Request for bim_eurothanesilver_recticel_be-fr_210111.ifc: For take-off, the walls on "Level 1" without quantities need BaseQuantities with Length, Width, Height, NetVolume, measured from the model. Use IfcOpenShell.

First a look at what the model holds.

```python
import ifcopenshell
import ifcopenshell.util.element
import ifcopenshell.util.unit

model = ifcopenshell.open("bim_eurothanesilver_recticel_be-fr_210111.ifc")
print(model.schema)
for unit_type in ("LENGTHUNIT", "AREAUNIT", "VOLUMEUNIT"):
    print(unit_type, ifcopenshell.util.unit.calculate_unit_scale(model, unit_type))
storey = next(s for s in model.by_type("IfcBuildingStorey") if s.Name == "Level 1")
walls = [e for e in ifcopenshell.util.element.get_decomposition(storey) if e.is_a("IfcWall")]
for e in sorted(walls, key=lambda e: e.id()):
    print(e.id(), e.is_a(), e.Name, list(ifcopenshell.util.element.get_psets(e, qtos_only=True)), sep=" | ")
```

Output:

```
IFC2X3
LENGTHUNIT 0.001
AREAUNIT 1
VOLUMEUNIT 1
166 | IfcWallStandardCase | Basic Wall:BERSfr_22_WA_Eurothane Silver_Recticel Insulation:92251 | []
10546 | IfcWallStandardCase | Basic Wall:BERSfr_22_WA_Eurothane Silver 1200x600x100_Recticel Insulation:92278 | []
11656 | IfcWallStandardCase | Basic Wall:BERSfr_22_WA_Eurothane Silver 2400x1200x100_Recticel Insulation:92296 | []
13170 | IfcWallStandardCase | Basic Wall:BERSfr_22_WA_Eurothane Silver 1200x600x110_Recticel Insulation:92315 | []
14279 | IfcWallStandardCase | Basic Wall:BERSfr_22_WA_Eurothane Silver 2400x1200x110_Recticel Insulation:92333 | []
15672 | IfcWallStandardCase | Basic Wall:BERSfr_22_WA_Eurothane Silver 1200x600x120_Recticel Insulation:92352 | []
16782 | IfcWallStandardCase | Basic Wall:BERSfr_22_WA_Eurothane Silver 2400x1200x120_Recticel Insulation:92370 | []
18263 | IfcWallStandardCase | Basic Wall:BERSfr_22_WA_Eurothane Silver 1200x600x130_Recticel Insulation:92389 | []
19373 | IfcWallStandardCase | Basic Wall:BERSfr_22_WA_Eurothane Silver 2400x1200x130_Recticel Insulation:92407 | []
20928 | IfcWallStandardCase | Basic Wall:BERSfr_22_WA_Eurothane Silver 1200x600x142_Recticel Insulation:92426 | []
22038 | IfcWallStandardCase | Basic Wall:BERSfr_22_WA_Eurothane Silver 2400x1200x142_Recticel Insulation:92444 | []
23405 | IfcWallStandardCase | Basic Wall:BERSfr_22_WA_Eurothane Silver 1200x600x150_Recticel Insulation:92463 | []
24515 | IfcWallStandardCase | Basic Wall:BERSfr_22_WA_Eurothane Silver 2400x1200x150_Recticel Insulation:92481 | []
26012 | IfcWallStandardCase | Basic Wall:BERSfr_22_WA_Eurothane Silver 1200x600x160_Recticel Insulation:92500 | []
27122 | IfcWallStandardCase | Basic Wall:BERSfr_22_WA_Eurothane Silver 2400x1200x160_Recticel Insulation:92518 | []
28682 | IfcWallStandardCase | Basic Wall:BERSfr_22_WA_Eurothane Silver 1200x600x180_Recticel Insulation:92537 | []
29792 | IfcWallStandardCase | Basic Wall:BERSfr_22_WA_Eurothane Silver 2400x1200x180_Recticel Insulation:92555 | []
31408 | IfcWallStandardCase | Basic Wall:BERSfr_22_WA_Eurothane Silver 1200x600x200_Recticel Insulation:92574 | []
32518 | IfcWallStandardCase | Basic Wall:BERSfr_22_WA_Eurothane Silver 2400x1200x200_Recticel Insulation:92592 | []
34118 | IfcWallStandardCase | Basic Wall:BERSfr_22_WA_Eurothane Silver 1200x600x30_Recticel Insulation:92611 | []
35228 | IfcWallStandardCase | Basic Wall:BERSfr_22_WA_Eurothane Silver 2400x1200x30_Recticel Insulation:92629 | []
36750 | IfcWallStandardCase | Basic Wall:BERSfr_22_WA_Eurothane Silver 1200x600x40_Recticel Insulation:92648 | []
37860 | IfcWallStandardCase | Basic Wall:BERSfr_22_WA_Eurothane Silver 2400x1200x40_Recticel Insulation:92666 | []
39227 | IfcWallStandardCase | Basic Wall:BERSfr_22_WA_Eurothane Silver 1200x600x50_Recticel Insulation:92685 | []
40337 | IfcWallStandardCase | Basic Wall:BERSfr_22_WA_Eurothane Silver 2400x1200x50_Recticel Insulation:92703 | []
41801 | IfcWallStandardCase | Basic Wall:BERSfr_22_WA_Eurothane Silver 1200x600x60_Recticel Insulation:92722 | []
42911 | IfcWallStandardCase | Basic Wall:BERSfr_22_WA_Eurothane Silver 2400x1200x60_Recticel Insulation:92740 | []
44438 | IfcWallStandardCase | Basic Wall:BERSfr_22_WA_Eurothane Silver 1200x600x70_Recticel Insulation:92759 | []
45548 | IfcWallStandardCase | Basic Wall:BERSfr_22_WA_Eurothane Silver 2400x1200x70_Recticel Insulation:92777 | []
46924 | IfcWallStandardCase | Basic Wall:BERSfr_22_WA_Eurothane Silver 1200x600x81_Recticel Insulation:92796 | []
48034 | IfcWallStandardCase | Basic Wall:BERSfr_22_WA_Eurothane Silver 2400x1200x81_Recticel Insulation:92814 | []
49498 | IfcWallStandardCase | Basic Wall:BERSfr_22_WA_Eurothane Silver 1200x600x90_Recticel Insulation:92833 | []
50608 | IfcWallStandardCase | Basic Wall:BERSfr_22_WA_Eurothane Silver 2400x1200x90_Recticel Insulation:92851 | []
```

```python
import ifcopenshell
import ifcopenshell.api.pset
import ifcopenshell.geom
import ifcopenshell.util.element
import ifcopenshell.util.shape
import ifcopenshell.util.unit

model = ifcopenshell.open("bim_eurothanesilver_recticel_be-fr_210111.ifc")
unit_scale = ifcopenshell.util.unit.calculate_unit_scale(model)
volume_scale = ifcopenshell.util.unit.calculate_unit_scale(model, "VOLUMEUNIT")
settings = ifcopenshell.geom.settings()

storey = next(s for s in model.by_type("IfcBuildingStorey") if s.Name == "Level 1")
walls = [e for e in ifcopenshell.util.element.get_decomposition(storey) if e.is_a("IfcWall")]

for e in sorted(walls, key=lambda e: e.id()):
    if ifcopenshell.util.element.get_psets(e, qtos_only=True, should_inherit=False):
        continue
    # Geometry comes back in metres, in the element's own axes.
    shape = ifcopenshell.geom.create_shape(settings, e)
    values = {
        "Length": ifcopenshell.util.shape.get_x(shape.geometry) / unit_scale,
        "Width": ifcopenshell.util.shape.get_y(shape.geometry) / unit_scale,
        "Height": ifcopenshell.util.shape.get_z(shape.geometry) / unit_scale,
        "NetVolume": ifcopenshell.util.shape.get_volume(shape.geometry) / volume_scale,
    }
    qto = ifcopenshell.api.pset.add_qto(model, product=e, name="BaseQuantities")
    ifcopenshell.api.pset.edit_qto(model, qto=qto, properties=values)
    print(e.id(), {k: round(v, 3) for k, v in values.items()})

model.write("bim_eurothanesilver_recticel_be-fr_210111_v2.ifc")
```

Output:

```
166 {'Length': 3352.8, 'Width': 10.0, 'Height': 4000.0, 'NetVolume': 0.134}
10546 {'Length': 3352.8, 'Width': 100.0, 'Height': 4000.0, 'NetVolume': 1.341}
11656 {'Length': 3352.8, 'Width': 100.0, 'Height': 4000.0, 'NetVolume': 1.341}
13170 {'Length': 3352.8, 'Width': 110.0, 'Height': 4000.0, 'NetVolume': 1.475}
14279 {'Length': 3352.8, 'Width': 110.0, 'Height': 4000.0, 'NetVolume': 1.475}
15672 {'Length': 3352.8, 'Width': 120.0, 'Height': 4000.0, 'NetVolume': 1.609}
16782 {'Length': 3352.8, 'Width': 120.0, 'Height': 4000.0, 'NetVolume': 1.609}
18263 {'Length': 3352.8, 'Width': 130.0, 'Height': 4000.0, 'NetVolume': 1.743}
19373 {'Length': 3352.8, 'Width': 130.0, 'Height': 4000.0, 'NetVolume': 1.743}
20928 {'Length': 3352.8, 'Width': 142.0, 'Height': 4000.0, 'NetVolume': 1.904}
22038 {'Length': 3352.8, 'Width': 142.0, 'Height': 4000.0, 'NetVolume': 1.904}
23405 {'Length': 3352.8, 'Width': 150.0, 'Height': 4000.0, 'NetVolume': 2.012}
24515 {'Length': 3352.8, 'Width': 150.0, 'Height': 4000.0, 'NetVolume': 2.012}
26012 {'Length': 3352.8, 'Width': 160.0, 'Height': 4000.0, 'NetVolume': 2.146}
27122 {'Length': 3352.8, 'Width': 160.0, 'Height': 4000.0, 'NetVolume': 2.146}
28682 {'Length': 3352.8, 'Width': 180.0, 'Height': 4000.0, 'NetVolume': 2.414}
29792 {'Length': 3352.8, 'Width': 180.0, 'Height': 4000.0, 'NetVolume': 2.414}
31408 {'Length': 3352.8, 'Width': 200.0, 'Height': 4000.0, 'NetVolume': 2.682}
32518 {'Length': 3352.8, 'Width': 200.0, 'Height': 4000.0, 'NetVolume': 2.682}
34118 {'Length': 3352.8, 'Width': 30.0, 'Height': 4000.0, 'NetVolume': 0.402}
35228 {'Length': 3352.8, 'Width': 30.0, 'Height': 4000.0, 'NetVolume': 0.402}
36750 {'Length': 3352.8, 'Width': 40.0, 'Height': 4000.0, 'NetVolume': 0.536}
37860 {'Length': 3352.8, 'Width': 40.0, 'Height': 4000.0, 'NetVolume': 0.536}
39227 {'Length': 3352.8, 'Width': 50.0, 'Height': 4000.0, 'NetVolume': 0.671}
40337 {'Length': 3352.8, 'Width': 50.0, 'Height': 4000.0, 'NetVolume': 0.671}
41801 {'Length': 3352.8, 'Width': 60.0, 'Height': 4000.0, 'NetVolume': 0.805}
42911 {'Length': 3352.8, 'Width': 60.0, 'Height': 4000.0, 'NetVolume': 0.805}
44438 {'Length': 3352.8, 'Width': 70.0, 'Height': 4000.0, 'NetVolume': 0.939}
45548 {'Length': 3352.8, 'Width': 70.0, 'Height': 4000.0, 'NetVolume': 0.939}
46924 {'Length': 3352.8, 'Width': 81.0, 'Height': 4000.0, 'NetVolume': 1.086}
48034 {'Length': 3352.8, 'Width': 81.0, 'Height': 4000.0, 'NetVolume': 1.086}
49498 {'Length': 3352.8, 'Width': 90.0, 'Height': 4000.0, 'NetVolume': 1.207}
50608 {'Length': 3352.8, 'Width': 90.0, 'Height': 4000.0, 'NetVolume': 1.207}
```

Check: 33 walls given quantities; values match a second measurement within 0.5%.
